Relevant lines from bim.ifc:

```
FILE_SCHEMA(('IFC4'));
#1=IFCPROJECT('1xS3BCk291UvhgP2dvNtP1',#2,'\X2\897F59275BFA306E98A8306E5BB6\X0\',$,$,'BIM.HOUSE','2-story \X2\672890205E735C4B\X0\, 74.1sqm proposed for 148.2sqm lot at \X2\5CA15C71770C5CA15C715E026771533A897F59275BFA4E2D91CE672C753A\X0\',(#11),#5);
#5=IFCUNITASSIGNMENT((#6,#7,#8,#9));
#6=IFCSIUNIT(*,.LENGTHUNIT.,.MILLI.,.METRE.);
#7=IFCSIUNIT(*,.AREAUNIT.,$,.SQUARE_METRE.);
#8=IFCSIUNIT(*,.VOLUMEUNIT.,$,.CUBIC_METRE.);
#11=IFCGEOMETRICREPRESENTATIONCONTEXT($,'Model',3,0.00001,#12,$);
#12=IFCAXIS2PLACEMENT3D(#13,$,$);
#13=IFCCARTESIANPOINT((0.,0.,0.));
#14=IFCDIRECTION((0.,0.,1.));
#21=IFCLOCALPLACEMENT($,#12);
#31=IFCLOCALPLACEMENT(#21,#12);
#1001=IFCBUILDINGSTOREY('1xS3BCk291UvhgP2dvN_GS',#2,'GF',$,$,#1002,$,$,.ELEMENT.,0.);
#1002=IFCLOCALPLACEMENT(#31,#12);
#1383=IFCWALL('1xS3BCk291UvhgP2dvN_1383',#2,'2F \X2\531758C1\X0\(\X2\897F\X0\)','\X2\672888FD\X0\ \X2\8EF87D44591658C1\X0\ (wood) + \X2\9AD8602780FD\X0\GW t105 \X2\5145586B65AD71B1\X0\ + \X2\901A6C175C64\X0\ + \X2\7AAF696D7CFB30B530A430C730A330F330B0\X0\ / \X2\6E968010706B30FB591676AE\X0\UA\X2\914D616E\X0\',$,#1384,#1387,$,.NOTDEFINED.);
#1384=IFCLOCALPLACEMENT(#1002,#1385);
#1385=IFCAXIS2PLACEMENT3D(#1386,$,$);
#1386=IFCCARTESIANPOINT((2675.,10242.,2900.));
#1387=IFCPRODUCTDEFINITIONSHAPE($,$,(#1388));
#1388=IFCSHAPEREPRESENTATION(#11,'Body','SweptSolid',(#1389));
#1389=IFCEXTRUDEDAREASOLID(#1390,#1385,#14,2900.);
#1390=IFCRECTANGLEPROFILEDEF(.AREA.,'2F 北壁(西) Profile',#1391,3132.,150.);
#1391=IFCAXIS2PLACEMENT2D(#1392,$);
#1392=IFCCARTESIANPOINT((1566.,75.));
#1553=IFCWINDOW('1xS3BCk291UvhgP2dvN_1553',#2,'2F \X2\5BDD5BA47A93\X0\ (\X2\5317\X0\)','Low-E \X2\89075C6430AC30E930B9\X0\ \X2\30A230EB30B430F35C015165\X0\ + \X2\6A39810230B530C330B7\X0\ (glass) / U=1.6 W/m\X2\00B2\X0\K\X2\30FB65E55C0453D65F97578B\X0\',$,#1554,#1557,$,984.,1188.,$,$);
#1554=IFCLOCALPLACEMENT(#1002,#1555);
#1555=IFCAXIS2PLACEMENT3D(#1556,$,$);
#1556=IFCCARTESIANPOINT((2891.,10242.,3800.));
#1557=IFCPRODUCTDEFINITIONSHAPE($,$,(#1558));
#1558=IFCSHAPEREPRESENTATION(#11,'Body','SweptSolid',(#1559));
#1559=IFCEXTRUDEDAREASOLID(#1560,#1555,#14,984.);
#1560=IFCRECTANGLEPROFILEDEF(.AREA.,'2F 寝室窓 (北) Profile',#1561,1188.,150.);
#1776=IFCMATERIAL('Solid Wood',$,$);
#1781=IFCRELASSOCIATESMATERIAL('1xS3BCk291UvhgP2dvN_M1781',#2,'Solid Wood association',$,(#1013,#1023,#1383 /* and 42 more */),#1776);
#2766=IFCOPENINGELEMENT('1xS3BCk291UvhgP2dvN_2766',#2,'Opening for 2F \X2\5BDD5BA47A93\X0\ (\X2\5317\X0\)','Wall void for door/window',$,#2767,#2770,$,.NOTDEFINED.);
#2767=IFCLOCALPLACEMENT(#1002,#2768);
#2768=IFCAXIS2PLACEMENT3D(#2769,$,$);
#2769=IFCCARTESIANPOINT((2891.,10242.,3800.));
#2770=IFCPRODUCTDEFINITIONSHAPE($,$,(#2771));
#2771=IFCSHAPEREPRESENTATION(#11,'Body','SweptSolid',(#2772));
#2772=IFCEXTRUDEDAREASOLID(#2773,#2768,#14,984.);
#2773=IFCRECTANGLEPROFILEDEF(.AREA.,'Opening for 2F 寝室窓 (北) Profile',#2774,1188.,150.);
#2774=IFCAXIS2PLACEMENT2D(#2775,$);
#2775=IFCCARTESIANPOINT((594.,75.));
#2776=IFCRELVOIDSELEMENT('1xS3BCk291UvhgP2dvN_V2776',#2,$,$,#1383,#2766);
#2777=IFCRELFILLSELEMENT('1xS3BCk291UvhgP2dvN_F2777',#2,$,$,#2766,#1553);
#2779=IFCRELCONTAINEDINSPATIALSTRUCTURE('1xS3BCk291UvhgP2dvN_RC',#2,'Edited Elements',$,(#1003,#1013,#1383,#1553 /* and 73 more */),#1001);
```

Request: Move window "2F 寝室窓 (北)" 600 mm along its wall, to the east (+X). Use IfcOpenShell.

```python
import ifcopenshell
import ifcopenshell.api.geometry
import ifcopenshell.util.placement
import ifcopenshell.util.unit

model = ifcopenshell.open("bim.ifc")
unit_scale = ifcopenshell.util.unit.calculate_unit_scale(model)

window = model.by_id(1553)
opening = window.FillsVoids[0].RelatingOpeningElement
wall = opening.VoidsElements[0].RelatingBuildingElement

wall_matrix = ifcopenshell.util.placement.get_local_placement(wall.ObjectPlacement)
shift = wall_matrix[:3, 0] * 0.6 / unit_scale
before = ifcopenshell.util.placement.get_local_placement(window.ObjectPlacement)[:3, 3].copy()

# The window is not placed relative to its opening, so move both.
for product in (opening, window):
    matrix = ifcopenshell.util.placement.get_local_placement(product.ObjectPlacement)
    matrix[:3, 3] += shift
    ifcopenshell.api.geometry.edit_object_placement(model, product=product, matrix=matrix, is_si=False)

after = ifcopenshell.util.placement.get_local_placement(window.ObjectPlacement)[:3, 3]
print("window moved by", (after - before).round(3) + 0.0)

model.write("bim_updated.ifc")
```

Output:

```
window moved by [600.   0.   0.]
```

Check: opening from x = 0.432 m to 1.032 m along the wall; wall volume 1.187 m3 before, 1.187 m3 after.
